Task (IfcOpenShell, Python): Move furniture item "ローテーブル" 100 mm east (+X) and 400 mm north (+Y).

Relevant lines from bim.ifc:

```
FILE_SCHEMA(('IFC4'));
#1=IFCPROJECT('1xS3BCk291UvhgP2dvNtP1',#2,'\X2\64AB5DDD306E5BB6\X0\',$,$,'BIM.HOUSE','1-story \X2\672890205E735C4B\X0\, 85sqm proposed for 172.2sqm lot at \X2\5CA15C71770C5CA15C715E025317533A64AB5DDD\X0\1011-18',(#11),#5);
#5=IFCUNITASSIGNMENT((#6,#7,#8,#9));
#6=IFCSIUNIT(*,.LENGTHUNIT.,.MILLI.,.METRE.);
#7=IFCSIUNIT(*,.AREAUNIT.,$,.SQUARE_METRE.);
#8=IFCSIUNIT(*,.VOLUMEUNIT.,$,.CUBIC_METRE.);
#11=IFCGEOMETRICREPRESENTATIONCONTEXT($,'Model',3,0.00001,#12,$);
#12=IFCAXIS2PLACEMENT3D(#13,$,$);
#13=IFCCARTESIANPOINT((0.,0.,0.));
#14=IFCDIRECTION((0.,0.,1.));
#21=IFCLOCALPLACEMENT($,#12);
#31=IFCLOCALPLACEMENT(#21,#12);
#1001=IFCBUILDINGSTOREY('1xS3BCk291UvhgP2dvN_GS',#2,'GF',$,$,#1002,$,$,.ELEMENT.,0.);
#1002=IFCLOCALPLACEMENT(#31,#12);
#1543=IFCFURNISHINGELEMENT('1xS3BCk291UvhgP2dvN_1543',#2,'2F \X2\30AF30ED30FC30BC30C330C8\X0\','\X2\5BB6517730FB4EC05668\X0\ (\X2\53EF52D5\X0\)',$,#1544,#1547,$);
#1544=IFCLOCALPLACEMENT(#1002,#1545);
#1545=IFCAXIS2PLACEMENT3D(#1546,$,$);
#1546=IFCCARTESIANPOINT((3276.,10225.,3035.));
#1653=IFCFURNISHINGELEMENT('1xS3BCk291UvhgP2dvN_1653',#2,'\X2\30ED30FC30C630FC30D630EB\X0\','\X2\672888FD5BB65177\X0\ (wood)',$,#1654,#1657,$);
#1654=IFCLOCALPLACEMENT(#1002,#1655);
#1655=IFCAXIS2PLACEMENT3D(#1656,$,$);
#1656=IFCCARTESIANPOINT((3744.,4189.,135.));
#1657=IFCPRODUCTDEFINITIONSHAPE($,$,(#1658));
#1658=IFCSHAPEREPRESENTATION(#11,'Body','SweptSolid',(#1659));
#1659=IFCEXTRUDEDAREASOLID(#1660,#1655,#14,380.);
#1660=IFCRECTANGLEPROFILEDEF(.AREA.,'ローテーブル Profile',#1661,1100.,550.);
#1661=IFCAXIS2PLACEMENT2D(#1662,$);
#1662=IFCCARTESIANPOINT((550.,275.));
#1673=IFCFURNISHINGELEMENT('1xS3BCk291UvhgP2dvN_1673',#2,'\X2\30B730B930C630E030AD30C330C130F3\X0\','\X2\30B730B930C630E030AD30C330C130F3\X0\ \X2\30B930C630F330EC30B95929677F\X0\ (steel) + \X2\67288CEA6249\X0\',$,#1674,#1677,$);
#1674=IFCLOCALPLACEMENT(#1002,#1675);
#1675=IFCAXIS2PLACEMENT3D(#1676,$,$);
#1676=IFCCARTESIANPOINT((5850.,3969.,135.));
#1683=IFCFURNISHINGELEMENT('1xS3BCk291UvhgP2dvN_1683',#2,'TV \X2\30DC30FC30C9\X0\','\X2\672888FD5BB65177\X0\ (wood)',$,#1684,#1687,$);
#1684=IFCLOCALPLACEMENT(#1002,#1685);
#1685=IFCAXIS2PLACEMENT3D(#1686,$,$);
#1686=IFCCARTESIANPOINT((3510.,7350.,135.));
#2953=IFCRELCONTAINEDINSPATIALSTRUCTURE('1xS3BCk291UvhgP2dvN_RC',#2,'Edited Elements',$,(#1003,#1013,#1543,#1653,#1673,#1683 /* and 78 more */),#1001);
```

```python
import ifcopenshell
import ifcopenshell.api.geometry
import ifcopenshell.util.placement

model = ifcopenshell.open("bim.ifc")

item = model.by_guid("1xS3BCk291UvhgP2dvN_1653")
matrix = ifcopenshell.util.placement.get_local_placement(item.ObjectPlacement)
matrix[0, 3] += 100.0
matrix[1, 3] += 400.0
ifcopenshell.api.geometry.edit_object_placement(model, product=item, matrix=matrix, is_si=False)

print(ifcopenshell.util.placement.get_local_placement(item.ObjectPlacement).round(3) + 0.0)

model.write("bim_edited.ifc")
```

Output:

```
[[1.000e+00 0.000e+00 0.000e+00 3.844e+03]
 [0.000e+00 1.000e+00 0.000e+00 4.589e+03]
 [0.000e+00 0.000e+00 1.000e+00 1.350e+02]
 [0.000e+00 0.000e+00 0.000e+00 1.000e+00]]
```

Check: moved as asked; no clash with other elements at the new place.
